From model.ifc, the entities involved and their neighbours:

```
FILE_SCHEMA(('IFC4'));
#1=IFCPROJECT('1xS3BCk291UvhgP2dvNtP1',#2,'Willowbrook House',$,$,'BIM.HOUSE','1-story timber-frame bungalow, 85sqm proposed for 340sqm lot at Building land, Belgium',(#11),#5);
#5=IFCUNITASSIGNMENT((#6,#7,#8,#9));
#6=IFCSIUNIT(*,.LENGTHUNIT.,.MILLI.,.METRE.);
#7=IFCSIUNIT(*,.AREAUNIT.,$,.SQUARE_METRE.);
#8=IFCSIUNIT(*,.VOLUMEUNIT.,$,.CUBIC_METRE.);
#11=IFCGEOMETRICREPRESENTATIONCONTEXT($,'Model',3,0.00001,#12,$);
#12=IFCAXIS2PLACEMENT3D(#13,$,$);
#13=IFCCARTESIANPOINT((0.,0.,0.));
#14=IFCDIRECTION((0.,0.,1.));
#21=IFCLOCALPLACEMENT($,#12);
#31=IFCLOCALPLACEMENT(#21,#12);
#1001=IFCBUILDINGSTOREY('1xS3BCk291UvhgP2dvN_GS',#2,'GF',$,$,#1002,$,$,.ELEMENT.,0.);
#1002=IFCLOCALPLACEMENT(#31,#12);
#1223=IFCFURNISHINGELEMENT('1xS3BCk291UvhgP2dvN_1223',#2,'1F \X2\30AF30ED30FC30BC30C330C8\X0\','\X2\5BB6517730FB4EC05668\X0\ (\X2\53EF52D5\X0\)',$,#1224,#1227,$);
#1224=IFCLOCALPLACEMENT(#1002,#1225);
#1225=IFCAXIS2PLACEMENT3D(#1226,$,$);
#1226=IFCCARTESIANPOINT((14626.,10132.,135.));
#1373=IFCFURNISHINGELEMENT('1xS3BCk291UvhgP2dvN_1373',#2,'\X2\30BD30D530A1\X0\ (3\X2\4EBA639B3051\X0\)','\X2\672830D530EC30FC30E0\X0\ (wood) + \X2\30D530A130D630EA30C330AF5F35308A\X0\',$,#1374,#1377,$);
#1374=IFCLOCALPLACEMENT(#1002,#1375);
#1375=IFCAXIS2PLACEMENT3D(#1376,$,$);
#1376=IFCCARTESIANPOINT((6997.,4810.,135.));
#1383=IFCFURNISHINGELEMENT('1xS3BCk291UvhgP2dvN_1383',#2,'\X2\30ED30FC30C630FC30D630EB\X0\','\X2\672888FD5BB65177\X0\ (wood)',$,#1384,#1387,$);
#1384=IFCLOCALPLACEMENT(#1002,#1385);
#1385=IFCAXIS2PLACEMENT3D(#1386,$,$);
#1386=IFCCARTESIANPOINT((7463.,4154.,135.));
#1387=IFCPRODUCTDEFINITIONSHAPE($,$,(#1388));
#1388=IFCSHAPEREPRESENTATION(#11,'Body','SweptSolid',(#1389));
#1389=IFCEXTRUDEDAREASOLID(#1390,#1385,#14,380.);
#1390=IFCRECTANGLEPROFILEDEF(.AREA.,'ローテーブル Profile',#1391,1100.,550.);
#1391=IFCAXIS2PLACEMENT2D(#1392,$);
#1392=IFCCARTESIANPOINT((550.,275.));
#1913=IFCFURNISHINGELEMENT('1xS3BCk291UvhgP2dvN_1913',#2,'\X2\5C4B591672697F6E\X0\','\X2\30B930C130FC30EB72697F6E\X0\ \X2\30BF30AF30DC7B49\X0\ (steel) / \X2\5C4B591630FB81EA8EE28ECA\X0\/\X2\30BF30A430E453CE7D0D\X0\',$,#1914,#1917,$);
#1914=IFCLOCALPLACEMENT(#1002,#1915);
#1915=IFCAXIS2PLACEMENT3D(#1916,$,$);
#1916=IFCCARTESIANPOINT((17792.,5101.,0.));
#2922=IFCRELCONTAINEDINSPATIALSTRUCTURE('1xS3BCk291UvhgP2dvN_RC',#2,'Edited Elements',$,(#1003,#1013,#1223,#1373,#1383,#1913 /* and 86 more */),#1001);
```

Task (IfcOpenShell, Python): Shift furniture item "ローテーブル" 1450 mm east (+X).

```python
import ifcopenshell
import ifcopenshell.api.geometry
import ifcopenshell.util.placement
import ifcopenshell.util.unit

model = ifcopenshell.open("model.ifc")
unit_scale = ifcopenshell.util.unit.calculate_unit_scale(model)

item = model.by_guid("1xS3BCk291UvhgP2dvN_1383")
matrix = ifcopenshell.util.placement.get_local_placement(item.ObjectPlacement)
matrix[0, 3] += 1.45 / unit_scale
ifcopenshell.api.geometry.edit_object_placement(model, product=item, matrix=matrix, is_si=False)

print(ifcopenshell.util.placement.get_local_placement(item.ObjectPlacement).round(3) + 0.0)

model.write("model_v2.ifc")
```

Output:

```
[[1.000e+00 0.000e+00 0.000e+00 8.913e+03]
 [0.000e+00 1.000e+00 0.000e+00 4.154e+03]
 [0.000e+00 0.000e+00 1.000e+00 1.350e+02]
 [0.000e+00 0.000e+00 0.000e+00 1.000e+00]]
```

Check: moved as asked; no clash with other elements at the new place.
